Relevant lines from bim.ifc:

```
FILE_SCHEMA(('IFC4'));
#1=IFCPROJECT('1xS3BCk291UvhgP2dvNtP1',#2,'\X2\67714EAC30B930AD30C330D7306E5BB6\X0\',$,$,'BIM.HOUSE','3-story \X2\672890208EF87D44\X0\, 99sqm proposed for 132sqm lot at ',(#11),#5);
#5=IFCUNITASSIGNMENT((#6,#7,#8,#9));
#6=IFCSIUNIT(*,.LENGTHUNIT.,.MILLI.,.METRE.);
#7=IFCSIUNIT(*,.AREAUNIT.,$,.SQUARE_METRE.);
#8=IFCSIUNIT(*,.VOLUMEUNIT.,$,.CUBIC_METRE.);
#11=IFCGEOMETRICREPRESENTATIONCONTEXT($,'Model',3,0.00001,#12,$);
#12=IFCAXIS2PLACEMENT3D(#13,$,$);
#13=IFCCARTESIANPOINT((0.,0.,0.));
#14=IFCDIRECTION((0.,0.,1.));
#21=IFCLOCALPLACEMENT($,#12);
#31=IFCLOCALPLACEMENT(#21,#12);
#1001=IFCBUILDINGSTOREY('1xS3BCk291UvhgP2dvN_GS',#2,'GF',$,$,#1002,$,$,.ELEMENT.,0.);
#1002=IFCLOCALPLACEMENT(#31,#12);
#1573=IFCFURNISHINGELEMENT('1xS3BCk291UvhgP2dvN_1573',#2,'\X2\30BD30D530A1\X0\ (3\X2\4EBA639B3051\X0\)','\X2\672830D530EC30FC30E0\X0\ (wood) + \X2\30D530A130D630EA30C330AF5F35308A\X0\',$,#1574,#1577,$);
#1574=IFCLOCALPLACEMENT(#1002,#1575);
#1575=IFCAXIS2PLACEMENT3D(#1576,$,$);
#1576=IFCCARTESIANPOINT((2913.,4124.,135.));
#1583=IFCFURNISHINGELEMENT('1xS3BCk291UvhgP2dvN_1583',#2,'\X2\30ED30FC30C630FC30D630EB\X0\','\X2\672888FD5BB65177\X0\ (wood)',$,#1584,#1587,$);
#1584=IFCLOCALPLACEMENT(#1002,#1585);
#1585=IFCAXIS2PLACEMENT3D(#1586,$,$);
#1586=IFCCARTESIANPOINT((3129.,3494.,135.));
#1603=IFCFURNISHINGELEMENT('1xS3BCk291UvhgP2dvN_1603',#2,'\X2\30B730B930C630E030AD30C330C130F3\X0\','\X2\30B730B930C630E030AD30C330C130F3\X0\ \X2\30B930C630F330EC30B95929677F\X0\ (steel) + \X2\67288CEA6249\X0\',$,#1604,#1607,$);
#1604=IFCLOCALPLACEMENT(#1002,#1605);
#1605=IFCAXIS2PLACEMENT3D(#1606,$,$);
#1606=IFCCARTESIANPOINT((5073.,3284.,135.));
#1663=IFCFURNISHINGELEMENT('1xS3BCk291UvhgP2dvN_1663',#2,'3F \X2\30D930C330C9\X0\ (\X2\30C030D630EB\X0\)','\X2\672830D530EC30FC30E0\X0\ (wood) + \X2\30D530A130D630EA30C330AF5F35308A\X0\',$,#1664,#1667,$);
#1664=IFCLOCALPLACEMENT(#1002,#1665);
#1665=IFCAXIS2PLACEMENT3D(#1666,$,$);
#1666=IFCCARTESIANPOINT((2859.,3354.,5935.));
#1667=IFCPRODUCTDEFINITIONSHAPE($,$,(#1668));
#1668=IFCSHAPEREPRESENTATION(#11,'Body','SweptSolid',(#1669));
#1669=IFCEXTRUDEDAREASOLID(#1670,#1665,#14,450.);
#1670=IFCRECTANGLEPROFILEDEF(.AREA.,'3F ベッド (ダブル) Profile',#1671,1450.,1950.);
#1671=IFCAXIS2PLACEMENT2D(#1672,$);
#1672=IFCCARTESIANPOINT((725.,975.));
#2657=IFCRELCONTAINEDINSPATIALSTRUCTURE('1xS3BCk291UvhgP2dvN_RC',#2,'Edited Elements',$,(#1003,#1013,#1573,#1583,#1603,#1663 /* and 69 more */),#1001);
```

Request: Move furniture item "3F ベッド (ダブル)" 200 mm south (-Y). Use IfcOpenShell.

```python
import ifcopenshell
import ifcopenshell.api.geometry
import ifcopenshell.util.placement
import ifcopenshell.util.unit

model = ifcopenshell.open("bim.ifc")
unit_scale = ifcopenshell.util.unit.calculate_unit_scale(model)

item = model.by_id(1663)
matrix = ifcopenshell.util.placement.get_local_placement(item.ObjectPlacement)
matrix[1, 3] -= 0.2 / unit_scale
ifcopenshell.api.geometry.edit_object_placement(model, product=item, matrix=matrix, is_si=False)

print(ifcopenshell.util.placement.get_local_placement(item.ObjectPlacement).round(3) + 0.0)

model.write("bim_updated.ifc")
```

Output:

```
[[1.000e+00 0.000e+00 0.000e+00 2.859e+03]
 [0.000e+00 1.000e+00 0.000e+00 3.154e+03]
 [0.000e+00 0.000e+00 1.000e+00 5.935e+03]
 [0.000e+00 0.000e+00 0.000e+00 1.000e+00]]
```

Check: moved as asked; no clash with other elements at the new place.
